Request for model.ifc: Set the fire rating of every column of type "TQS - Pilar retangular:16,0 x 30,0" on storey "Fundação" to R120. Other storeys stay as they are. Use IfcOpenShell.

First a look at what the model holds.

```python
import ifcopenshell
import ifcopenshell.util.element

model = ifcopenshell.open("model.ifc")
print(model.schema)
storey = next(s for s in model.by_type("IfcBuildingStorey") if s.Name == "Fundação")
columns = [e for e in ifcopenshell.util.element.get_decomposition(storey) if e.is_a("IfcColumn")]
seen = {}
for e in columns:
    element_type = ifcopenshell.util.element.get_type(e)
    key = (element_type.Name if element_type != e and element_type else None, ifcopenshell.util.element.get_pset(e, "Pset_ColumnCommon", "FireRating"))
    seen[key] = seen.get(key, 0) + 1
for (name, value), count in sorted(seen.items(), key=str):
    print(count, "x", name, "|", value)
```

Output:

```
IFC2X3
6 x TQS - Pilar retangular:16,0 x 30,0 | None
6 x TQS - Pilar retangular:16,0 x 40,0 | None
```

```python
import ifcopenshell
import ifcopenshell.api.pset
import ifcopenshell.util.element

model = ifcopenshell.open("model.ifc")

storey = next(s for s in model.by_type("IfcBuildingStorey") if s.Name == "Fundação")
columns = [e for e in ifcopenshell.util.element.get_decomposition(storey) if e.is_a("IfcColumn")]

count = 0
for e in columns:
    element_type = ifcopenshell.util.element.get_type(e)
    if element_type in (None, e) or element_type.Name != "TQS - Pilar retangular:16,0 x 30,0":
        continue
    # add_pset returns the element's existing set when there is one.
    pset = ifcopenshell.api.pset.add_pset(model, product=e, name="Pset_ColumnCommon")
    ifcopenshell.api.pset.edit_pset(model, pset=pset, properties={"FireRating": "R120"})
    count += 1

print(count, "columns updated")

model.write("model_edited.ifc")
```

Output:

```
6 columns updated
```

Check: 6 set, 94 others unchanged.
